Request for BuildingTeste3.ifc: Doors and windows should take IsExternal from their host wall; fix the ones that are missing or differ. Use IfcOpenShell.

First a look at what the model holds.

```python
import ifcopenshell
import ifcopenshell.util.element

model = ifcopenshell.open("BuildingTeste3.ifc")
print(model.schema)
seen = {}
for e in model.by_type("IfcDoor") + model.by_type("IfcWindow"):
    if not e.FillsVoids:
        continue
    host = e.FillsVoids[0].RelatingOpeningElement.VoidsElements[0].RelatingBuildingElement
    own = ifcopenshell.util.element.get_pset(e, f"Pset_{e.is_a()[3:].removesuffix('StandardCase')}Common", "IsExternal")
    wall = ifcopenshell.util.element.get_pset(host, "Pset_WallCommon", "IsExternal")
    seen[e.is_a(), own, wall] = seen.get((e.is_a(), own, wall), 0) + 1
for (cls, own, wall), count in sorted(seen.items(), key=str):
    print(count, cls, "IsExternal:", own, "| host wall:", wall)
```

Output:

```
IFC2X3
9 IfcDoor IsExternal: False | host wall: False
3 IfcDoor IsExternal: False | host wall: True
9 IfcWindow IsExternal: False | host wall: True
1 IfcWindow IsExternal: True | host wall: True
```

```python
import ifcopenshell
import ifcopenshell.api.pset
import ifcopenshell.util.element

model = ifcopenshell.open("BuildingTeste3.ifc")

count = 0
for ifc_class, pset_name in (("IfcDoor", "Pset_DoorCommon"), ("IfcWindow", "Pset_WindowCommon")):
    for e in model.by_type(ifc_class):
        if not e.FillsVoids:
            continue
        host = e.FillsVoids[0].RelatingOpeningElement.VoidsElements[0].RelatingBuildingElement
        external = ifcopenshell.util.element.get_pset(host, "Pset_WallCommon", "IsExternal")
        if external is None or ifcopenshell.util.element.get_pset(e, pset_name, "IsExternal") == external:
            continue
        pset = ifcopenshell.api.pset.add_pset(model, product=e, name=pset_name)
        ifcopenshell.api.pset.edit_pset(model, pset=pset, properties={"IsExternal": external})
        count += 1

print(count, "updated")

model.write("BuildingTeste3-out.ifc")
```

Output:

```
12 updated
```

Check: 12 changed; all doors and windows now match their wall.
